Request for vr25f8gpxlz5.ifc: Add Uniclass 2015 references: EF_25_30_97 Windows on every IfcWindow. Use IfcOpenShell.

First a look at what the model holds.

```python
import ifcopenshell

model = ifcopenshell.open("vr25f8gpxlz5.ifc")
print(model.schema)
print("classifications:", [c.Name for c in model.by_type("IfcClassification")])
for ifc_class in ("IfcDoor", "IfcRoof", "IfcStair", "IfcWall", "IfcWindow"):
    print(ifc_class, len(model.by_type(ifc_class)))
```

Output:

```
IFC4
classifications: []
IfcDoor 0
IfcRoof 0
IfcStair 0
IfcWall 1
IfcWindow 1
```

```python
import ifcopenshell
import ifcopenshell.api.classification

model = ifcopenshell.open("vr25f8gpxlz5.ifc")

system = ifcopenshell.api.classification.add_classification(model, classification="Uniclass 2015")

codes = {
    "IfcWindow": ("EF_25_30_97", "Windows"),
}
for ifc_class, (code, name) in codes.items():
    products = model.by_type(ifc_class)
    ifcopenshell.api.classification.add_reference(
        model, products=products, classification=system, identification=code, name=name
    )
    print(code, len(products))

model.write("vr25f8gpxlz5_rev.ifc")
```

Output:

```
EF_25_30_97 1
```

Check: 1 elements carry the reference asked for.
